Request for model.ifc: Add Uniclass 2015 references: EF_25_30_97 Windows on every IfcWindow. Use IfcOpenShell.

First a look at what the model holds.

```python
import ifcopenshell

model = ifcopenshell.open("model.ifc")
print(model.schema)
print("classifications:", [c.Name for c in model.by_type("IfcClassification")])
for ifc_class in ("IfcDoor", "IfcRoof", "IfcStair", "IfcWall", "IfcWindow"):
    print(ifc_class, len(model.by_type(ifc_class)))
```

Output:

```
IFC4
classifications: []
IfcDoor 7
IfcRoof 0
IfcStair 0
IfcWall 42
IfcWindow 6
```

```python
import ifcopenshell
import ifcopenshell.api.classification

model = ifcopenshell.open("model.ifc")

system = ifcopenshell.api.classification.add_classification(model, classification="Uniclass 2015")

codes = {
    "IfcWindow": ("EF_25_30_97", "Windows"),
}
for ifc_class, (code, name) in codes.items():
    products = model.by_type(ifc_class)
    ifcopenshell.api.classification.add_reference(
        model, products=products, classification=system, identification=code, name=name
    )
    print(code, len(products))

model.write("model_rev.ifc")
```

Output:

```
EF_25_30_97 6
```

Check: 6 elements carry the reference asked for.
